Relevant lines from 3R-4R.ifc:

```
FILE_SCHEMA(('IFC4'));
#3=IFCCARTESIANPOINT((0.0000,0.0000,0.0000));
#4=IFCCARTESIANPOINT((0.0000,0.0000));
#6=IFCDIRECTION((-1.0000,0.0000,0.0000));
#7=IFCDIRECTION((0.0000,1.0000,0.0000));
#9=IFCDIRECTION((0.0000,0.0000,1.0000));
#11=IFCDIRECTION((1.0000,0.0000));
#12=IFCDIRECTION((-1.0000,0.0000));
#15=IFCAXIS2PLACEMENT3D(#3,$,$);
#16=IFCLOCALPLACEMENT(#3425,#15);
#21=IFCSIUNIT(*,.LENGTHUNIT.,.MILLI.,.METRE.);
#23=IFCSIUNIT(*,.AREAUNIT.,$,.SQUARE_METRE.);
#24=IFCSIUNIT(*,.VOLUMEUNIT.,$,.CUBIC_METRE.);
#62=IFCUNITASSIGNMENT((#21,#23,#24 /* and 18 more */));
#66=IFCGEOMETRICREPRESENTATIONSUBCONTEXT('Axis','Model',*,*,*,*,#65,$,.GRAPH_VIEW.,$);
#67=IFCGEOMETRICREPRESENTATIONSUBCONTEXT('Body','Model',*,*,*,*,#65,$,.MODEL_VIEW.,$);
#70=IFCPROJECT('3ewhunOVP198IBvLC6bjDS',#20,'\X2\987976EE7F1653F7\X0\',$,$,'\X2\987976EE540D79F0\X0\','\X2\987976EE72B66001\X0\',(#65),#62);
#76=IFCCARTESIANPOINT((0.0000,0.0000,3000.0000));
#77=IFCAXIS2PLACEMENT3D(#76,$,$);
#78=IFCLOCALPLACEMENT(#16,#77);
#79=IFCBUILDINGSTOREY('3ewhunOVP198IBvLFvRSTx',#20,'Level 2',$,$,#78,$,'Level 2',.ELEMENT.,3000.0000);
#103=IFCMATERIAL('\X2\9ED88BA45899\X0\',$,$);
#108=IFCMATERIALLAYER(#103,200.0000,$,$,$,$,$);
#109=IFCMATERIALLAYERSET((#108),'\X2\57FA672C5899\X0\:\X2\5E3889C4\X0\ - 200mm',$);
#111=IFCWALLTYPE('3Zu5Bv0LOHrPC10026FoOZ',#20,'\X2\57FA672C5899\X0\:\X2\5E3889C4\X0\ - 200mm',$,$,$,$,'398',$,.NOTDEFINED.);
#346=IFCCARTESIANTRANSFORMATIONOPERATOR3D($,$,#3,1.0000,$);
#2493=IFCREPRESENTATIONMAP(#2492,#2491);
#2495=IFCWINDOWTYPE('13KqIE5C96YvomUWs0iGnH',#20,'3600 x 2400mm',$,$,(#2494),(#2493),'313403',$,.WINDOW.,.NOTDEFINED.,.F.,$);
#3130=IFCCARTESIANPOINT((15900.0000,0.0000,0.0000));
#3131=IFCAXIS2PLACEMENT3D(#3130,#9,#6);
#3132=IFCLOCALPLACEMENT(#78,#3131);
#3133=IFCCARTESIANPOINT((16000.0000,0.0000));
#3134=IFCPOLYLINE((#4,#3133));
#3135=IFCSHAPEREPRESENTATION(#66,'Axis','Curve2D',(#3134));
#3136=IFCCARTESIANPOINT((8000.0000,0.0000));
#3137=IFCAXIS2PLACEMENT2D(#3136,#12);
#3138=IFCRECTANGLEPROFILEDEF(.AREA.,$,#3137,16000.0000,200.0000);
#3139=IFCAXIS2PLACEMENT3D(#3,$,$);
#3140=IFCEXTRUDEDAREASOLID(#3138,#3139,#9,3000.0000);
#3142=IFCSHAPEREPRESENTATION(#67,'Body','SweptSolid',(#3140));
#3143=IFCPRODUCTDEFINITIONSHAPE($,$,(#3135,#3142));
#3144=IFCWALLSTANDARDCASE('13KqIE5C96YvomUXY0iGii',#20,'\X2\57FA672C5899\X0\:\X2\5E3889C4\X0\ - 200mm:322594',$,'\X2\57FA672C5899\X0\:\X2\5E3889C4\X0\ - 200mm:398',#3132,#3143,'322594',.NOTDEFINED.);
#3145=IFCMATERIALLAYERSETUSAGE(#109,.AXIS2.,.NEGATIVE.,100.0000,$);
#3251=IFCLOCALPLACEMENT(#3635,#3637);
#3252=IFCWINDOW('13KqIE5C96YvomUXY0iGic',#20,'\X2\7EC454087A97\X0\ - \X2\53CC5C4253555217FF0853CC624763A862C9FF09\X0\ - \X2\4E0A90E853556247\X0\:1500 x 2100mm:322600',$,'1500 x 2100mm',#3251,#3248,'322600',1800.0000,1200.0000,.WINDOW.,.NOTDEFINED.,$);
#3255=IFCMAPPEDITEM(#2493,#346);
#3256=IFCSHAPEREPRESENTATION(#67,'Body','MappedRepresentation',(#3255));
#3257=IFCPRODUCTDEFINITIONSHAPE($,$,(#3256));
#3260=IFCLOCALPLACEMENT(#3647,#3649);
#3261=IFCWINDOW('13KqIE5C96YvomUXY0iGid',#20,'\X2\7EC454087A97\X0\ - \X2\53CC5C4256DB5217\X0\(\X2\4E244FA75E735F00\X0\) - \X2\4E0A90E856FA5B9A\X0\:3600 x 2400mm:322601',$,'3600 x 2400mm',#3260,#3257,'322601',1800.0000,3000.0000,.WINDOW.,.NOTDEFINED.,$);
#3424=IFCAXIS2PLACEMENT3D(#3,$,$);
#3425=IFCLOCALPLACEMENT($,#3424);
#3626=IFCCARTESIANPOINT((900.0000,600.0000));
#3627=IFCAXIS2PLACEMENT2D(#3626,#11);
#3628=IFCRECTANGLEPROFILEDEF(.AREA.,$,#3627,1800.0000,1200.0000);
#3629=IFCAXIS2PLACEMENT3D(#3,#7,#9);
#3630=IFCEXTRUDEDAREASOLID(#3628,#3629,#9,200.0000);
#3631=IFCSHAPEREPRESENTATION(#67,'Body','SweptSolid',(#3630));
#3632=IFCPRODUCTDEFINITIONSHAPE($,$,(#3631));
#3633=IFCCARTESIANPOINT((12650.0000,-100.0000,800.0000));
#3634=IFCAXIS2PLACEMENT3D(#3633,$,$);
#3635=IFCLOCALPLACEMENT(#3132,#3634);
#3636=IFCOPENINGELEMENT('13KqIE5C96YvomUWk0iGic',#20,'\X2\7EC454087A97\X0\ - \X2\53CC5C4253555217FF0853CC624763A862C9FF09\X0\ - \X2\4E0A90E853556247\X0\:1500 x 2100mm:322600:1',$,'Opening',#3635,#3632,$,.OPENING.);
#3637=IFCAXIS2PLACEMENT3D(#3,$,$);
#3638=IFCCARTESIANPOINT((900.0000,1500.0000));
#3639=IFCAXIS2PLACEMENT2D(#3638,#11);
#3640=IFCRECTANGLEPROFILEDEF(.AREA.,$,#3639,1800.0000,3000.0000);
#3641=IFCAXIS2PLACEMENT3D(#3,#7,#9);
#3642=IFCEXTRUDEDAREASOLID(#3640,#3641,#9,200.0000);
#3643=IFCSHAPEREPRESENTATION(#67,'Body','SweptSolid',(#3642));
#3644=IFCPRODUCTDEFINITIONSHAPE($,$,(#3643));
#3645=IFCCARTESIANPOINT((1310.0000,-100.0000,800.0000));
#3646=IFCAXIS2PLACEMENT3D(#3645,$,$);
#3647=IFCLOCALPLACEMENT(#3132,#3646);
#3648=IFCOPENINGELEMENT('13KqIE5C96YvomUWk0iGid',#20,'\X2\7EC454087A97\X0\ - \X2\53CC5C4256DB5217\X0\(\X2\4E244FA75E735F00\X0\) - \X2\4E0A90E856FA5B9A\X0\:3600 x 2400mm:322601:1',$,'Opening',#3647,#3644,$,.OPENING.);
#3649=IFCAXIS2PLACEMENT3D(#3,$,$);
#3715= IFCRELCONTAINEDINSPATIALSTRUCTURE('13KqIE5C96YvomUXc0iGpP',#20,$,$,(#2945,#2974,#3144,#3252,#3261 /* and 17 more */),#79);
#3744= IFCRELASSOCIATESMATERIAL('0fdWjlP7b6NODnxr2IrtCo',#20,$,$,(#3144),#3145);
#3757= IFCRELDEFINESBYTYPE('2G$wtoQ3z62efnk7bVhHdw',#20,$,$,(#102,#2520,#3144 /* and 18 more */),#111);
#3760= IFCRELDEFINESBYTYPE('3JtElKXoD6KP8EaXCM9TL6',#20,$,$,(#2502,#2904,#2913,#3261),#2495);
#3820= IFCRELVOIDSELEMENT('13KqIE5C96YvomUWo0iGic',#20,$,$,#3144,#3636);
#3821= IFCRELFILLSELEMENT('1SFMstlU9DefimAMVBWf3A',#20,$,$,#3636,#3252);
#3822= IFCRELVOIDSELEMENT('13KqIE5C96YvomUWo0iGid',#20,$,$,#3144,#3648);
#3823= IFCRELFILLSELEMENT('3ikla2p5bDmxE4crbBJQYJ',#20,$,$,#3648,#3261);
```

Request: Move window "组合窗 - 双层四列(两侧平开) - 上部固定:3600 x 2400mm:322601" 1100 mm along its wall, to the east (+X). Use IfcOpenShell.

```python
import ifcopenshell
import ifcopenshell.api.geometry
import ifcopenshell.util.placement

model = ifcopenshell.open("3R-4R.ifc")

window = model.by_guid("13KqIE5C96YvomUXY0iGid")
opening = window.FillsVoids[0].RelatingOpeningElement
wall = opening.VoidsElements[0].RelatingBuildingElement

wall_matrix = ifcopenshell.util.placement.get_local_placement(wall.ObjectPlacement)
shift = wall_matrix[:3, 0] * -1100.0
before = ifcopenshell.util.placement.get_local_placement(window.ObjectPlacement)[:3, 3].copy()

# The window is placed relative to its opening, so it follows when the opening moves.
matrix = ifcopenshell.util.placement.get_local_placement(opening.ObjectPlacement)
matrix[:3, 3] += shift
ifcopenshell.api.geometry.edit_object_placement(
    model, product=opening, matrix=matrix, is_si=False, should_transform_children=True
)

after = ifcopenshell.util.placement.get_local_placement(window.ObjectPlacement)[:3, 3]
print("window moved by", (after - before).round(3) + 0.0)

model.write("3R-4R-out.ifc")
```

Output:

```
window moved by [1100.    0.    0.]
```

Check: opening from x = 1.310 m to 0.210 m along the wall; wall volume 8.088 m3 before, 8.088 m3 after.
